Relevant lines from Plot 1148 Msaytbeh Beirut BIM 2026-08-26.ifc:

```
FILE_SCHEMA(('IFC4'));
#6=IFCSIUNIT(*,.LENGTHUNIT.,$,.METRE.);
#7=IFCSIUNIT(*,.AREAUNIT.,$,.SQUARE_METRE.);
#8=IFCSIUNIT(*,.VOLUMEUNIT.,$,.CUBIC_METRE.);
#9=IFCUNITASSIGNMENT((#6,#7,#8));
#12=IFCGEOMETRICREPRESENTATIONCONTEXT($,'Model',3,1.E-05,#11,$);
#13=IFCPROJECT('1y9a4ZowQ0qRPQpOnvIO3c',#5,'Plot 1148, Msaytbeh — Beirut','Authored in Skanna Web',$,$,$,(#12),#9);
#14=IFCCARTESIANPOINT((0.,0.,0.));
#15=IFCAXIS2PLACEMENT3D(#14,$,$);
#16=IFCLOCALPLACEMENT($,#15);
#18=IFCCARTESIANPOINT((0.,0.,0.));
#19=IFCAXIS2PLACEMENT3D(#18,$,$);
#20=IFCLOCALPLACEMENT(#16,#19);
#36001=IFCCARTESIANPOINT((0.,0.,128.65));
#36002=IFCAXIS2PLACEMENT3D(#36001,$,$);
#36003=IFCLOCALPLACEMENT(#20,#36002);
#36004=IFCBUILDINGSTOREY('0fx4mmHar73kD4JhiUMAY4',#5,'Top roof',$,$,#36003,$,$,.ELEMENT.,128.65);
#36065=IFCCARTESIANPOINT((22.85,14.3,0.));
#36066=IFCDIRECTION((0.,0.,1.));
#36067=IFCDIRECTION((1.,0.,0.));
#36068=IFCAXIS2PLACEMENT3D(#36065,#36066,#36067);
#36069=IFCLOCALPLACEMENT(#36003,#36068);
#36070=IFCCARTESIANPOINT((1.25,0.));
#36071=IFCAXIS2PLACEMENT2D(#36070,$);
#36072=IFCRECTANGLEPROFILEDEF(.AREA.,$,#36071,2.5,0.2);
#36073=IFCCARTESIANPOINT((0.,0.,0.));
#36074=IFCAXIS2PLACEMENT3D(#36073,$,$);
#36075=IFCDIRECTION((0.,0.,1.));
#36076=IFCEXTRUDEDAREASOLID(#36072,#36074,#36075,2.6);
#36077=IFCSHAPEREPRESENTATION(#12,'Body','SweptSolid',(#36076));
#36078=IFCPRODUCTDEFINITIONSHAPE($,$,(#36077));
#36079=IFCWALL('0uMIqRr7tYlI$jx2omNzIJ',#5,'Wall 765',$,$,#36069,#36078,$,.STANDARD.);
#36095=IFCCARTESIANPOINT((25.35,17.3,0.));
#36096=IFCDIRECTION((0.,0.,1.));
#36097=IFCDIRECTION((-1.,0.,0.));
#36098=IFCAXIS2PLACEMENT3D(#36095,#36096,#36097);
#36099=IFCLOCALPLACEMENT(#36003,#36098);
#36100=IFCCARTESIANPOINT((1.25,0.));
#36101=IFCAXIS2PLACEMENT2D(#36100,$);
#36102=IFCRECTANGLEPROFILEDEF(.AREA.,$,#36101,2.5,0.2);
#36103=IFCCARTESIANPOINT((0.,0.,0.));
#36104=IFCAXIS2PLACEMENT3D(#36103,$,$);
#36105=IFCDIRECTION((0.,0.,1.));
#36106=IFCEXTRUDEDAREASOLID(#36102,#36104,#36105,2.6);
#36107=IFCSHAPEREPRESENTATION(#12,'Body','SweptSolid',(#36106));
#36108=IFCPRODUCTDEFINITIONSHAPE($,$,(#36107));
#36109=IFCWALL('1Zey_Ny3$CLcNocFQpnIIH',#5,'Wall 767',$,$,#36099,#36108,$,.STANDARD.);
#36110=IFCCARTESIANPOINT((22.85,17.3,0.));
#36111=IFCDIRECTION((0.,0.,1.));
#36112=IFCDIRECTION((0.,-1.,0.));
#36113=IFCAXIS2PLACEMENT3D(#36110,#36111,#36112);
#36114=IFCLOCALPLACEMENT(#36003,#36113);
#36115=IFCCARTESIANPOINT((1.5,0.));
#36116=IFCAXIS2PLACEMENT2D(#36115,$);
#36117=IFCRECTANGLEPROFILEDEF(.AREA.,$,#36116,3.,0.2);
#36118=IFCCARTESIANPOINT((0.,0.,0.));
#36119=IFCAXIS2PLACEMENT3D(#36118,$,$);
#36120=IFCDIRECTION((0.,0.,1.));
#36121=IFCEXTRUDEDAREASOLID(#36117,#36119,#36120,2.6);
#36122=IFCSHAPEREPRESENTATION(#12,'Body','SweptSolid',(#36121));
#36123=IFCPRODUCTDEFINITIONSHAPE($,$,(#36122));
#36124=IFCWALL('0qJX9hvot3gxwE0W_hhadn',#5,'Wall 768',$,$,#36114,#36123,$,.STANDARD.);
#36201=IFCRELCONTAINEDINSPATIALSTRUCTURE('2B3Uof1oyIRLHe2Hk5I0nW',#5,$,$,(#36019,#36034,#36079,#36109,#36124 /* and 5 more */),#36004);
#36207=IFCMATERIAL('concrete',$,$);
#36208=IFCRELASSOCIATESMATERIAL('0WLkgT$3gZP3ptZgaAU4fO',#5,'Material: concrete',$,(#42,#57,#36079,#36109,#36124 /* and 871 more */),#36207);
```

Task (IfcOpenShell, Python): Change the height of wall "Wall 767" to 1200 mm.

```python
import ifcopenshell
import ifcopenshell.geom
import ifcopenshell.util.shape
import ifcopenshell.util.unit

model = ifcopenshell.open("Plot 1148 Msaytbeh Beirut BIM 2026-08-26.ifc")
unit_scale = ifcopenshell.util.unit.calculate_unit_scale(model)
settings = ifcopenshell.geom.settings()


def volume(element):
    """Net volume in cubic metres, openings subtracted."""
    shape = ifcopenshell.geom.create_shape(settings, element)
    return ifcopenshell.util.shape.get_volume(shape.geometry)


wall = model.by_guid("1Zey_Ny3$CLcNocFQpnIIH")
before = volume(wall)

body = next(r for r in wall.Representation.Representations if r.RepresentationIdentifier == "Body")
solid = body.Items[0]
old_height = solid.Depth
solid.Depth = 1.2 / unit_scale
after = volume(wall)

print(f"height {old_height:g} -> {solid.Depth:g}, volume {before:.3f} -> {after:.3f} m3")

model.write("Plot 1148 Msaytbeh Beirut BIM 2026-08-26-out.ifc")
```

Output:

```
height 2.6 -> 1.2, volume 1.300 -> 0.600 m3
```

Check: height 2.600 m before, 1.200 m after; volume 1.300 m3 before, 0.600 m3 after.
